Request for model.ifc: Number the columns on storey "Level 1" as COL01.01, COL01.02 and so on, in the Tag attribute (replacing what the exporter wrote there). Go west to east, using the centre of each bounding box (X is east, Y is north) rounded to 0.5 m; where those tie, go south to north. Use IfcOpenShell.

First a look at what the model holds.

```python
import ifcopenshell
import ifcopenshell.util.element
import ifcopenshell.util.placement

model = ifcopenshell.open("model.ifc")
print(model.schema)
storey = next(s for s in model.by_type("IfcBuildingStorey") if s.Name == "Level 1")
columns = [e for e in ifcopenshell.util.element.get_decomposition(storey) if e.is_a("IfcColumn")]
for e in sorted(columns, key=lambda e: e.id()):
    origin = ifcopenshell.util.placement.get_local_placement(e.ObjectPlacement)[:3, 3]
    print(e.id(), e.Tag, e.Name, origin.round(2) + 0.0, sep=" | ")
```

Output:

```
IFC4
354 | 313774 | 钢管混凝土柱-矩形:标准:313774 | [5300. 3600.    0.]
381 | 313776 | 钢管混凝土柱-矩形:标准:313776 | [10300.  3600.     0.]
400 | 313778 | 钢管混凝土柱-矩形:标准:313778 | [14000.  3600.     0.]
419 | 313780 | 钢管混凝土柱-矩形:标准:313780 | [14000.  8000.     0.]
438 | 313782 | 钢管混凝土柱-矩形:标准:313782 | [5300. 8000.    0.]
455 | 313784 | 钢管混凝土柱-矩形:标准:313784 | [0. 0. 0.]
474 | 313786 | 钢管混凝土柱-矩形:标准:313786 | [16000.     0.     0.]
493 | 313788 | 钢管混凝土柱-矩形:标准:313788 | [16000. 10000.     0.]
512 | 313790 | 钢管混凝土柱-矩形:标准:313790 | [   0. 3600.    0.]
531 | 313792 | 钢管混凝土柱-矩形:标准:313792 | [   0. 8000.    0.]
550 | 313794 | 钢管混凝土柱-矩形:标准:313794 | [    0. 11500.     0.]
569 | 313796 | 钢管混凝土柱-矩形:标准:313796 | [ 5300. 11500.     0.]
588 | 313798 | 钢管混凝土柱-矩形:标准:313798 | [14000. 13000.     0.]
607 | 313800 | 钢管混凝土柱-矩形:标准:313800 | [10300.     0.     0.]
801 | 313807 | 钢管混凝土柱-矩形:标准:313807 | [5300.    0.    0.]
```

```python
import ifcopenshell
import ifcopenshell.geom
import ifcopenshell.util.element
import ifcopenshell.util.shape

model = ifcopenshell.open("model.ifc")
settings = ifcopenshell.geom.settings()
settings.set("use-world-coords", True)


def centre(element):
    shape = ifcopenshell.geom.create_shape(settings, element)
    return ifcopenshell.util.shape.get_bbox_centroid(shape.geometry)


storey = next(s for s in model.by_type("IfcBuildingStorey") if s.Name == "Level 1")
columns = [e for e in ifcopenshell.util.element.get_decomposition(storey) if e.is_a("IfcColumn")]

# Insertion points can sit at a corner or the storey origin, so sort by the geometry (in metres).
centres = {e: centre(e) for e in columns}
columns.sort(key=lambda e: (round(centres[e][0] / 0.5), centres[e][1]))

for i, e in enumerate(columns, start=1):
    number = f"COL01.{i:02d}"
    e.Tag = number
    print(e.id(), number)

model.write("model-out.ifc")
```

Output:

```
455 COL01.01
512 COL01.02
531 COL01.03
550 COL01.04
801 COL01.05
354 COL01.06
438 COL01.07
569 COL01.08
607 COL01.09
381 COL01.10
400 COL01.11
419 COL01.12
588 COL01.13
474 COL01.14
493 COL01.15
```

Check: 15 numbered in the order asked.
